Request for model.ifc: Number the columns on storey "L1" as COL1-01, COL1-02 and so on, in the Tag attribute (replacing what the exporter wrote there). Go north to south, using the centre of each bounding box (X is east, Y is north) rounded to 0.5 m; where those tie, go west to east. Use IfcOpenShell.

First a look at what the model holds.

```python
import ifcopenshell
import ifcopenshell.util.element
import ifcopenshell.util.placement

model = ifcopenshell.open("model.ifc")
print(model.schema)
storey = next(s for s in model.by_type("IfcBuildingStorey") if s.Name == "L1")
columns = [e for e in ifcopenshell.util.element.get_decomposition(storey) if e.is_a("IfcColumn")]
for e in sorted(columns, key=lambda e: e.id()):
    origin = ifcopenshell.util.placement.get_local_placement(e.ObjectPlacement)[:3, 3]
    print(e.id(), e.Tag, e.Name, origin.round(2) + 0.0, sep=" | ")
```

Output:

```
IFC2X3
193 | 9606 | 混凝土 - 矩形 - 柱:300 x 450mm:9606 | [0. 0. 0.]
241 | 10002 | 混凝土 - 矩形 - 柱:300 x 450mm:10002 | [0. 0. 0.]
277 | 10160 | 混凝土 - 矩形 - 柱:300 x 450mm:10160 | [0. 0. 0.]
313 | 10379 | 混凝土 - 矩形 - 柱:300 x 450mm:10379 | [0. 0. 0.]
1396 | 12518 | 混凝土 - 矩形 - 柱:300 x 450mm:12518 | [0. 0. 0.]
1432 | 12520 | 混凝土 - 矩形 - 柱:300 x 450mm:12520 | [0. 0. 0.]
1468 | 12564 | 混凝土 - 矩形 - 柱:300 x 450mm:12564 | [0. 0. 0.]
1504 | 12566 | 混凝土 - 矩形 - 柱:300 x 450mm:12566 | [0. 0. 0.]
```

```python
import ifcopenshell
import ifcopenshell.geom
import ifcopenshell.util.element
import ifcopenshell.util.shape

model = ifcopenshell.open("model.ifc")
settings = ifcopenshell.geom.settings()
settings.set("use-world-coords", True)


def centre(element):
    shape = ifcopenshell.geom.create_shape(settings, element)
    return ifcopenshell.util.shape.get_bbox_centroid(shape.geometry)


storey = next(s for s in model.by_type("IfcBuildingStorey") if s.Name == "L1")
columns = [e for e in ifcopenshell.util.element.get_decomposition(storey) if e.is_a("IfcColumn")]

# Insertion points can sit at a corner or the storey origin, so sort by the geometry (in metres).
centres = {e: centre(e) for e in columns}
columns.sort(key=lambda e: (-round(centres[e][1] / 0.5), centres[e][0]))

for i, e in enumerate(columns, start=1):
    number = f"COL1-{i:02d}"
    e.Tag = number
    print(e.id(), number)

model.write("model_edited.ifc")
```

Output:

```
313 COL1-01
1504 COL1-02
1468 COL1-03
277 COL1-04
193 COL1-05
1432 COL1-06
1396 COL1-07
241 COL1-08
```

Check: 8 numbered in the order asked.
